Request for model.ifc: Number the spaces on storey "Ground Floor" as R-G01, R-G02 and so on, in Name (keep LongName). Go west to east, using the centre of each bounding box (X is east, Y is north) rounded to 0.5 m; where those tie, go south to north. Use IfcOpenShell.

First a look at what the model holds.

```python
import ifcopenshell
import ifcopenshell.util.element
import ifcopenshell.util.placement

model = ifcopenshell.open("model.ifc")
print(model.schema)
storey = next(s for s in model.by_type("IfcBuildingStorey") if s.Name == "Ground Floor")
spaces = [e for e in ifcopenshell.util.element.get_decomposition(storey) if e.is_a("IfcSpace")]
for e in sorted(spaces, key=lambda e: e.id()):
    origin = ifcopenshell.util.placement.get_local_placement(e.ObjectPlacement)[:3, 3]
    print(e.id(), e.Name, e.LongName, origin.round(2) + 0.0, sep=" | ")
```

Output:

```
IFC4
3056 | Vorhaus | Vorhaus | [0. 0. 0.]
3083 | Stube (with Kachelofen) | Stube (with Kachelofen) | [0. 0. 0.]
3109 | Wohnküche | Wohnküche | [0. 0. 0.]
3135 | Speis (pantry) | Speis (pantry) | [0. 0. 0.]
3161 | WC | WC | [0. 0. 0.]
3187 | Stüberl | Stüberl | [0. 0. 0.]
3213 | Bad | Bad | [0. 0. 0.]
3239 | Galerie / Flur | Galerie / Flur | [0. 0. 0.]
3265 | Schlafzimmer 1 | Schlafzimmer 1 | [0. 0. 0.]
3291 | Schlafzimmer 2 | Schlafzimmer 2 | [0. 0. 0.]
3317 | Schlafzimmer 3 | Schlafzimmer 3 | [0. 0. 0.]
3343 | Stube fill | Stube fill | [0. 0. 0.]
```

```python
import ifcopenshell
import ifcopenshell.geom
import ifcopenshell.util.element
import ifcopenshell.util.shape

model = ifcopenshell.open("model.ifc")
settings = ifcopenshell.geom.settings()
settings.set("use-world-coords", True)


def centre(element):
    shape = ifcopenshell.geom.create_shape(settings, element)
    return ifcopenshell.util.shape.get_bbox_centroid(shape.geometry)


storey = next(s for s in model.by_type("IfcBuildingStorey") if s.Name == "Ground Floor")
spaces = [e for e in ifcopenshell.util.element.get_decomposition(storey) if e.is_a("IfcSpace")]

# Insertion points can sit at a corner or the storey origin, so sort by the geometry (in metres).
centres = {e: centre(e) for e in spaces}
spaces.sort(key=lambda e: (round(centres[e][0] / 0.5), centres[e][1]))

for i, e in enumerate(spaces, start=1):
    number = f"R-G{i:02d}"
    e.Name = number
    print(e.id(), number)

model.write("model-out.ifc")
```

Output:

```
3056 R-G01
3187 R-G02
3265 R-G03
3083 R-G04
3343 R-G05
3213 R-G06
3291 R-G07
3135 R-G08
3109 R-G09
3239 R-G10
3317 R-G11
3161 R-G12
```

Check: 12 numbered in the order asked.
